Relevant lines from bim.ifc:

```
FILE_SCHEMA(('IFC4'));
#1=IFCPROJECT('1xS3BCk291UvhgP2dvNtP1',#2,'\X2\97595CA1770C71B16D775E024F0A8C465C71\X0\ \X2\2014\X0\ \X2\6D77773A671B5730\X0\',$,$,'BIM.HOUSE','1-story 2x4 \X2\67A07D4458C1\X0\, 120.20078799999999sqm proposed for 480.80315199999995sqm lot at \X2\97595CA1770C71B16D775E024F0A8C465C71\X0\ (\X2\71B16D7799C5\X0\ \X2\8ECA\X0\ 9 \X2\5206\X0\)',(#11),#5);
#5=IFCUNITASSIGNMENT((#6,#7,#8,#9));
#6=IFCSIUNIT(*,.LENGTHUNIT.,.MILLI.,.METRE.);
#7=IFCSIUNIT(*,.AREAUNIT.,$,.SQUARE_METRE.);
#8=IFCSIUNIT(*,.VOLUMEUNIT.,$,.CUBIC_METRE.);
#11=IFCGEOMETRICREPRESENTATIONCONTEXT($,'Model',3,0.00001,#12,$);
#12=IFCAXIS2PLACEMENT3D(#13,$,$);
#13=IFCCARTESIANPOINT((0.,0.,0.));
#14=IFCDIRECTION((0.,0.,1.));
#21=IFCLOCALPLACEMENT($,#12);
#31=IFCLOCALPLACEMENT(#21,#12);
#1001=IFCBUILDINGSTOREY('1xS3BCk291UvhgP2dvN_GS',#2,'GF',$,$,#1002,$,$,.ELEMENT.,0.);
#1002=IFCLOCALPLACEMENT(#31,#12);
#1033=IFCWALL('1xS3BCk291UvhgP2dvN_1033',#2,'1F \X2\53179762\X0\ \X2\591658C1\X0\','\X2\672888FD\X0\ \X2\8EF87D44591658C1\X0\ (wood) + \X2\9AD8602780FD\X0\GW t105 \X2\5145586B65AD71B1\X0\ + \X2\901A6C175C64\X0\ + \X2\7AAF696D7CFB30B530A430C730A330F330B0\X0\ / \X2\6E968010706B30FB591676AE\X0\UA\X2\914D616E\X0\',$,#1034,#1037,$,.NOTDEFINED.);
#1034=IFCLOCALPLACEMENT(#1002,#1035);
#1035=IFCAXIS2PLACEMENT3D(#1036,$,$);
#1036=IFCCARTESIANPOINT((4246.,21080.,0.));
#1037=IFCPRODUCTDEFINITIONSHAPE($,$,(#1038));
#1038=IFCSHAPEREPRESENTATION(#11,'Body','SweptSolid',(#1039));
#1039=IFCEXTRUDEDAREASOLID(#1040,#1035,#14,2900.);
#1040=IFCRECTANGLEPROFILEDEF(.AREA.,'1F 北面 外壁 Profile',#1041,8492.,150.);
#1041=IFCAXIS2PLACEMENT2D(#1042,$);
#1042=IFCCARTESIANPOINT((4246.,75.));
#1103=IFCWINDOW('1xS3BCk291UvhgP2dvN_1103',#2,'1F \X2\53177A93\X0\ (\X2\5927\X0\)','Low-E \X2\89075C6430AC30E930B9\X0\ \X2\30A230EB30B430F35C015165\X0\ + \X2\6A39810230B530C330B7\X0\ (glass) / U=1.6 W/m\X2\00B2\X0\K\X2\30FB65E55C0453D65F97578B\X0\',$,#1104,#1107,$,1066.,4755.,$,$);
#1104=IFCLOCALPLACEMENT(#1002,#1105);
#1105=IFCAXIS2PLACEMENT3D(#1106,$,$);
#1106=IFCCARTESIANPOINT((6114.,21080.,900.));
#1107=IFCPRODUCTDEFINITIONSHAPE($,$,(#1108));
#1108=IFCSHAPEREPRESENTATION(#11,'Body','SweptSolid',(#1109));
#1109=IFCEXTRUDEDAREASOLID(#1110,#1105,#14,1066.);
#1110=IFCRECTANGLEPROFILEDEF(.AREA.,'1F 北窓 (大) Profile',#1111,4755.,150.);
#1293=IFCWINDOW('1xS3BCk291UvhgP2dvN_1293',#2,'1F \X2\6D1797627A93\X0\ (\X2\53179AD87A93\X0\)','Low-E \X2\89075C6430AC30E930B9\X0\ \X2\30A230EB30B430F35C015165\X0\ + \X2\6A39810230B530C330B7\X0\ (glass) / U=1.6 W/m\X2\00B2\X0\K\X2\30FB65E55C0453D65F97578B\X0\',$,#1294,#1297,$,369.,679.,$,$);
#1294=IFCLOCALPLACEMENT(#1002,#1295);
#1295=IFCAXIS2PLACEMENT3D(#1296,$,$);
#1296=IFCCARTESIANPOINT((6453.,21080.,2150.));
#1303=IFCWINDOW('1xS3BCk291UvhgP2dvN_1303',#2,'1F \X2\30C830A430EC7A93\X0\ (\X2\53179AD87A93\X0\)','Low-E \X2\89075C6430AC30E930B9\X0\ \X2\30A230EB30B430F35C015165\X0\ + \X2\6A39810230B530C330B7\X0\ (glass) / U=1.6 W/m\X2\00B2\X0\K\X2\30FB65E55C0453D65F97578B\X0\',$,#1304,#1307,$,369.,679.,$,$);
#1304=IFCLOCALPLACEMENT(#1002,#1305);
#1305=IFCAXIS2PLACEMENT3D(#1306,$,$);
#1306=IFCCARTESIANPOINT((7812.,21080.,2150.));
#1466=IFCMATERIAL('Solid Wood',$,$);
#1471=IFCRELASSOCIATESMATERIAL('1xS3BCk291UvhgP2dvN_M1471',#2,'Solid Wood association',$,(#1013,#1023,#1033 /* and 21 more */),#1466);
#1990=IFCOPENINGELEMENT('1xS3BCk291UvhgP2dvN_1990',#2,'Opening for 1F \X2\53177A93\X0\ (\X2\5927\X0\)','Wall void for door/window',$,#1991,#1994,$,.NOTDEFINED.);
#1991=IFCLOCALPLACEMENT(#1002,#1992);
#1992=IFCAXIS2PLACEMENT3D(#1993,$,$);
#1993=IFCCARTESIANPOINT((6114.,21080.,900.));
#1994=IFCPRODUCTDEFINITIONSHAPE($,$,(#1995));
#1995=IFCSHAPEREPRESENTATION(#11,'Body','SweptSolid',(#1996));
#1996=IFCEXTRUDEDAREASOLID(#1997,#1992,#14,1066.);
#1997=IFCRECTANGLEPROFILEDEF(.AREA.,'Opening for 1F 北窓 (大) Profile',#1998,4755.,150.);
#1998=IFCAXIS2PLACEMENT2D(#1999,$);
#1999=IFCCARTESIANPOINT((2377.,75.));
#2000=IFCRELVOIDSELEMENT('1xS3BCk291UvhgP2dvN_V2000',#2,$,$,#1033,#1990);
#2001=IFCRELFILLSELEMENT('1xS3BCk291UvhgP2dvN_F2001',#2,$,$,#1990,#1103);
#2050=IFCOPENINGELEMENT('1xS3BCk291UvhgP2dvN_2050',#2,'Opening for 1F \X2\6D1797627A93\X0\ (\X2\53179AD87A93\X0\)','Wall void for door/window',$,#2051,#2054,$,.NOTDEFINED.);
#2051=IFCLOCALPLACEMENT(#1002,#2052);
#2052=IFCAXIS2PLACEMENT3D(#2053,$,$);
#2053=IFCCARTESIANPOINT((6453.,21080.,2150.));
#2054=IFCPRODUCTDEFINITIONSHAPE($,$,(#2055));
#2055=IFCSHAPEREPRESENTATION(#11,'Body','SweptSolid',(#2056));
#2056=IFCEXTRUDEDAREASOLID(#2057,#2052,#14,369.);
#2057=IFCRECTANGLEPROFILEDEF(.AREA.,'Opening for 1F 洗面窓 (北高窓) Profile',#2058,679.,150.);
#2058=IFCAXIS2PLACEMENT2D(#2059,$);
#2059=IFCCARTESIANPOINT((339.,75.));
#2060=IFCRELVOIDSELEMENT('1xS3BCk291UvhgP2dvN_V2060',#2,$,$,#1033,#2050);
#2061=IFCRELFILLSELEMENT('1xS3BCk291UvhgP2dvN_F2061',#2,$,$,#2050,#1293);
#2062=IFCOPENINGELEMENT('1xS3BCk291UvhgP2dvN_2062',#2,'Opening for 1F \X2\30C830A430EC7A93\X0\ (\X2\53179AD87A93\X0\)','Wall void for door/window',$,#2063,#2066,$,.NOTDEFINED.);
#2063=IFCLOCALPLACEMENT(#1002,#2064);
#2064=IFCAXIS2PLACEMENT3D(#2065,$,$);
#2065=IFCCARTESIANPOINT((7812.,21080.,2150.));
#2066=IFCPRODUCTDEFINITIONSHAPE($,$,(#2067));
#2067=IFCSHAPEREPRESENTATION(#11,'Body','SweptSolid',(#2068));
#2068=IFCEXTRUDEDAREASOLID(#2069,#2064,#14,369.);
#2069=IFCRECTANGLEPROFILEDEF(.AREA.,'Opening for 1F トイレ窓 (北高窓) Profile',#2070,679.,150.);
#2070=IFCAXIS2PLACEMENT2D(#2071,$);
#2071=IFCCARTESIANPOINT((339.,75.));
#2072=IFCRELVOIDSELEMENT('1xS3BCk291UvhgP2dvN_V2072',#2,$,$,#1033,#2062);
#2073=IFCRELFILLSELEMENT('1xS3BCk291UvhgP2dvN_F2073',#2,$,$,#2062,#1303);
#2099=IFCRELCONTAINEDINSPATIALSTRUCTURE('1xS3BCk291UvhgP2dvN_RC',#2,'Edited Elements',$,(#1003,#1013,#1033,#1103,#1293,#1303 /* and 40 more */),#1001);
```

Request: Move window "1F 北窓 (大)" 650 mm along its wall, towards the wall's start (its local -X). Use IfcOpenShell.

```python
import ifcopenshell
import ifcopenshell.api.geometry
import ifcopenshell.util.placement
import ifcopenshell.util.unit

model = ifcopenshell.open("bim.ifc")
unit_scale = ifcopenshell.util.unit.calculate_unit_scale(model)

window = model.by_guid("1xS3BCk291UvhgP2dvN_1103")
opening = window.FillsVoids[0].RelatingOpeningElement
wall = opening.VoidsElements[0].RelatingBuildingElement

wall_matrix = ifcopenshell.util.placement.get_local_placement(wall.ObjectPlacement)
shift = wall_matrix[:3, 0] * -0.65 / unit_scale
before = ifcopenshell.util.placement.get_local_placement(window.ObjectPlacement)[:3, 3].copy()

# The window is not placed relative to its opening, so move both.
for product in (opening, window):
    matrix = ifcopenshell.util.placement.get_local_placement(product.ObjectPlacement)
    matrix[:3, 3] += shift
    ifcopenshell.api.geometry.edit_object_placement(model, product=product, matrix=matrix, is_si=False)

after = ifcopenshell.util.placement.get_local_placement(window.ObjectPlacement)[:3, 3]
print("window moved by", (after - before).round(3) + 0.0)

model.write("bim_rev.ifc")
```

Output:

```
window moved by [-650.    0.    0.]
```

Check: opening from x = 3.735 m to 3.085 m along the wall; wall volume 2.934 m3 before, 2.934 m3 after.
